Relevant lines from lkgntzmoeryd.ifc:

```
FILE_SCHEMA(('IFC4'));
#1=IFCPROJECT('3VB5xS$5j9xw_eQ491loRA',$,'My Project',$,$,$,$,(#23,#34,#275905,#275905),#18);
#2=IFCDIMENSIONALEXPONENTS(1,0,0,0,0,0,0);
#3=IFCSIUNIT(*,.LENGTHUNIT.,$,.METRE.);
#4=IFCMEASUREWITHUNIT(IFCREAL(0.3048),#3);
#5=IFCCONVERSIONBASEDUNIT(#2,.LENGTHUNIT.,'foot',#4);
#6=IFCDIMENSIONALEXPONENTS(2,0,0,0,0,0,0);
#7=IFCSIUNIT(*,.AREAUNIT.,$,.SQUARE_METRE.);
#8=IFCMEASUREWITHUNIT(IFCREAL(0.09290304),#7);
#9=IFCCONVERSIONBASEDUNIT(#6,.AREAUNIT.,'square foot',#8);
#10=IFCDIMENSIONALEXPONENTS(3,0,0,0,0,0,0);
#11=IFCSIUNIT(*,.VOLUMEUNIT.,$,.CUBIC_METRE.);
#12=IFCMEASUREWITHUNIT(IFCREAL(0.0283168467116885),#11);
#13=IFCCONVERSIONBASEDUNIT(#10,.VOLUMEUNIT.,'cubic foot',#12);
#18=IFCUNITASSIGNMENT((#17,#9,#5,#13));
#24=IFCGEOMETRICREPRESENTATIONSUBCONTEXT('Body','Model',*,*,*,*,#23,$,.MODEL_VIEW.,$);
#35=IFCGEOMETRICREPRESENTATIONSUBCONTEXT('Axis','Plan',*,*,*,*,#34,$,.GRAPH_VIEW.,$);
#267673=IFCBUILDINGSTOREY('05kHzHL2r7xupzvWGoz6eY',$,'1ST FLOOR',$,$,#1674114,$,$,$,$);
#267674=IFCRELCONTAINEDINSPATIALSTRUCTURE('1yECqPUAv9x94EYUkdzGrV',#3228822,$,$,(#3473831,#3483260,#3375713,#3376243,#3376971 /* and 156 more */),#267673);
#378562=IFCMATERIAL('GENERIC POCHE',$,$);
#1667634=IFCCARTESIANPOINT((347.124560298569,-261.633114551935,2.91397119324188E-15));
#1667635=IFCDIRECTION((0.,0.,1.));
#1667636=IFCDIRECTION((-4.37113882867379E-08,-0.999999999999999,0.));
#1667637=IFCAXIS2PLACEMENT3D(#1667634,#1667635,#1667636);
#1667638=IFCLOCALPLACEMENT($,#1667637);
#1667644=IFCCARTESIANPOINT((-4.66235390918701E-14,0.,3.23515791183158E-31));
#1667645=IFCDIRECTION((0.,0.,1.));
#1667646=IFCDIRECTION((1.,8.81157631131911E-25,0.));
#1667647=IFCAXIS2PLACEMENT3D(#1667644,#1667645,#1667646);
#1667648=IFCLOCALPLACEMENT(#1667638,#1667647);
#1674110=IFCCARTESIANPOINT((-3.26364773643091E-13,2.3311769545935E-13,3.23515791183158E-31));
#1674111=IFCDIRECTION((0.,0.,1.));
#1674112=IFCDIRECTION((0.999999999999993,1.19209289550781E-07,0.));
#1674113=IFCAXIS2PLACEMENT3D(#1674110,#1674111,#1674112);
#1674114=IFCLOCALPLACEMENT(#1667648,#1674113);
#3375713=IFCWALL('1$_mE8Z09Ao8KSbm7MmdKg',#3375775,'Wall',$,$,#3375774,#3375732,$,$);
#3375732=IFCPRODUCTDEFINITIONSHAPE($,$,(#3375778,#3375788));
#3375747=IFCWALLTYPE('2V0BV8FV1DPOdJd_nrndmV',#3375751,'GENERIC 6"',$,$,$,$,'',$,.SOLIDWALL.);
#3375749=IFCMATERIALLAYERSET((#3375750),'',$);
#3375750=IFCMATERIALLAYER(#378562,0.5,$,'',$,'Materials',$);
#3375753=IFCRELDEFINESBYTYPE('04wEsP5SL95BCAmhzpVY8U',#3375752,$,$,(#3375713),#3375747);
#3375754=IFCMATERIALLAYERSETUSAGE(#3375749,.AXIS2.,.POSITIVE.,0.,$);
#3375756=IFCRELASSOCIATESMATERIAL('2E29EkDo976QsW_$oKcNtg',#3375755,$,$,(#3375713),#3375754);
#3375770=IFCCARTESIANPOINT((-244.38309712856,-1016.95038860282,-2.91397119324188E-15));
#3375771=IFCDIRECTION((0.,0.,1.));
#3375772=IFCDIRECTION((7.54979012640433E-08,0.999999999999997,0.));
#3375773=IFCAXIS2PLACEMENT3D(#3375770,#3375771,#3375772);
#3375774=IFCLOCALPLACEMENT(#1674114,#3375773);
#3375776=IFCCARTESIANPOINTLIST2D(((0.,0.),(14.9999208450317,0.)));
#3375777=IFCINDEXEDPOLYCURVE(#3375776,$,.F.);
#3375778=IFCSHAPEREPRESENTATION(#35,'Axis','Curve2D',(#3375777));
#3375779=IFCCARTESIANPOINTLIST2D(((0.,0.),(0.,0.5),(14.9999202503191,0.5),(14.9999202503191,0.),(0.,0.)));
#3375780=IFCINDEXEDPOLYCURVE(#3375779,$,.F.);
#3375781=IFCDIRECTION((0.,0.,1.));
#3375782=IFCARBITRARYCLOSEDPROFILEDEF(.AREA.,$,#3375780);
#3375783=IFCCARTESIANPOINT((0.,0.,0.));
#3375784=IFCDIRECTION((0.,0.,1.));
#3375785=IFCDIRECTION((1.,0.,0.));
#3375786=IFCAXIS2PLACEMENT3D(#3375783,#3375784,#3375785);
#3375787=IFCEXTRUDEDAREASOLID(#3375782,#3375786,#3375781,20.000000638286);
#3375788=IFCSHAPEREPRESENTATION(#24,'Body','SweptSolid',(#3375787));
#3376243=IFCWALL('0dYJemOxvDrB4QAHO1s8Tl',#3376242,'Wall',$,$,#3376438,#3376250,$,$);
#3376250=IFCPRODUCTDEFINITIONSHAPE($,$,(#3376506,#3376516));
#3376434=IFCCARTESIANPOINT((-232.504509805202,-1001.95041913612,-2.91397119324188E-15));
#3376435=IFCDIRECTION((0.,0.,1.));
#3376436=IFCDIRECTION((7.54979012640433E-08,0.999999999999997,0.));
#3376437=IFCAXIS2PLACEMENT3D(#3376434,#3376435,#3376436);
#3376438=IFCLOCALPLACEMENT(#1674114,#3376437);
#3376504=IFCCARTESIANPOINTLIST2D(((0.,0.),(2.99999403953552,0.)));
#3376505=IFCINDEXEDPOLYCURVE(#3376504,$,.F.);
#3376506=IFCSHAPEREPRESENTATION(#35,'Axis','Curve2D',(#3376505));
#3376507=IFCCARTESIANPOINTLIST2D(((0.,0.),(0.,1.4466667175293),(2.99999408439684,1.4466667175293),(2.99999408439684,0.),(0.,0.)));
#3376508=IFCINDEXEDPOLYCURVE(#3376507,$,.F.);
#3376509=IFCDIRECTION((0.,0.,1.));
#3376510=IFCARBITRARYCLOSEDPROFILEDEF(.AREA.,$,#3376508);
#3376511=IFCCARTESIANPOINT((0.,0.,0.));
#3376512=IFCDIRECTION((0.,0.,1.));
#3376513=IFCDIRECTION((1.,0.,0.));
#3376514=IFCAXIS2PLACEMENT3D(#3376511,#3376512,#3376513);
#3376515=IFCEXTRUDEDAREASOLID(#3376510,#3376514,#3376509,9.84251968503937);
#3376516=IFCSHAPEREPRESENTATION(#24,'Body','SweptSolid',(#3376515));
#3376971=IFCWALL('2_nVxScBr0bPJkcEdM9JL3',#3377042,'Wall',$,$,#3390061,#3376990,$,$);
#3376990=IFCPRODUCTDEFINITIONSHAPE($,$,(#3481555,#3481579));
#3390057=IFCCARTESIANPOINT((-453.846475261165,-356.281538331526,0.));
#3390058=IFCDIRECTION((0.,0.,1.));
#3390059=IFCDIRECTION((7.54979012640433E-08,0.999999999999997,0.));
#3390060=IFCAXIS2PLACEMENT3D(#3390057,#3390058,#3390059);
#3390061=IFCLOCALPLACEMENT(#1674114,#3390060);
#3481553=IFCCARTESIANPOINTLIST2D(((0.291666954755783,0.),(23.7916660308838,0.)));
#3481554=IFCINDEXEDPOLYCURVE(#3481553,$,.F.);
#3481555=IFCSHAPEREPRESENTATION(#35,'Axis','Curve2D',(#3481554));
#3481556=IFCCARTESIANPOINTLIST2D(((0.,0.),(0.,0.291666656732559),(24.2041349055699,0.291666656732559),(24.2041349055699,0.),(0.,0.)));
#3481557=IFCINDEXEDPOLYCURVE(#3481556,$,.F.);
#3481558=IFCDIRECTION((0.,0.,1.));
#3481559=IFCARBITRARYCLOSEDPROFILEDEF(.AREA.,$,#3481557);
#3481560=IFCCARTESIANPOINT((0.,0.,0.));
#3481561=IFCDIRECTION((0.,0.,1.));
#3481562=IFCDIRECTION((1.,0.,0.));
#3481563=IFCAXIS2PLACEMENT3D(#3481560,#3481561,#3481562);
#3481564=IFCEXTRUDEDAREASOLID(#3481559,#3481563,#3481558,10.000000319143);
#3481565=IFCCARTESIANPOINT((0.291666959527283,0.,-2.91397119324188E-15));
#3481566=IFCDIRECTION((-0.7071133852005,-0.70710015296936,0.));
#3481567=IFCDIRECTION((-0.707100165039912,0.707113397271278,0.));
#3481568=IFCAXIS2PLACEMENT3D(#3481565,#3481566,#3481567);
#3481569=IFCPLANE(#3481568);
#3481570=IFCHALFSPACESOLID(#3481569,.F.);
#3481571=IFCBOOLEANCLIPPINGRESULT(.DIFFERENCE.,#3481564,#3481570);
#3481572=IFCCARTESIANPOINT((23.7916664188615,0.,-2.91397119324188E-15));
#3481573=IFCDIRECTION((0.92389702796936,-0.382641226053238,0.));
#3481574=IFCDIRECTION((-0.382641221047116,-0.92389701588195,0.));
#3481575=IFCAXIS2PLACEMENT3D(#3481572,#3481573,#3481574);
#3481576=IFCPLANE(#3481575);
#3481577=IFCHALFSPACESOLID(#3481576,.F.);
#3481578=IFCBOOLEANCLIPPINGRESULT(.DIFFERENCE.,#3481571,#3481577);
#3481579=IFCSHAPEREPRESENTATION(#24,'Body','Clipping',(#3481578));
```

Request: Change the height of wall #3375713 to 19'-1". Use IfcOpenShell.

```python
import ifcopenshell
import ifcopenshell.geom
import ifcopenshell.util.representation
import ifcopenshell.util.shape
import ifcopenshell.util.unit

model = ifcopenshell.open("lkgntzmoeryd.ifc")
unit_scale = ifcopenshell.util.unit.calculate_unit_scale(model)
settings = ifcopenshell.geom.settings()


def volume(element):
    """Net volume in cubic metres, openings subtracted."""
    shape = ifcopenshell.geom.create_shape(settings, element)
    return ifcopenshell.util.shape.get_volume(shape.geometry)


wall = model.by_guid("1$_mE8Z09Ao8KSbm7MmdKg")
before = volume(wall)

body = ifcopenshell.util.representation.get_representation(wall, "Model", "Body")
solid = body.Items[0]
old_height = solid.Depth
solid.Depth = 229 * 0.0254 / unit_scale
after = volume(wall)

print(f"height {old_height:g} -> {solid.Depth:g}, volume {before:.3f} -> {after:.3f} m3")

model.write("lkgntzmoeryd-out.ifc")
```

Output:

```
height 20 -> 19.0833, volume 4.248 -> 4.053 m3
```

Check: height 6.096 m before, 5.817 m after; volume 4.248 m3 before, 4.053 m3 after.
